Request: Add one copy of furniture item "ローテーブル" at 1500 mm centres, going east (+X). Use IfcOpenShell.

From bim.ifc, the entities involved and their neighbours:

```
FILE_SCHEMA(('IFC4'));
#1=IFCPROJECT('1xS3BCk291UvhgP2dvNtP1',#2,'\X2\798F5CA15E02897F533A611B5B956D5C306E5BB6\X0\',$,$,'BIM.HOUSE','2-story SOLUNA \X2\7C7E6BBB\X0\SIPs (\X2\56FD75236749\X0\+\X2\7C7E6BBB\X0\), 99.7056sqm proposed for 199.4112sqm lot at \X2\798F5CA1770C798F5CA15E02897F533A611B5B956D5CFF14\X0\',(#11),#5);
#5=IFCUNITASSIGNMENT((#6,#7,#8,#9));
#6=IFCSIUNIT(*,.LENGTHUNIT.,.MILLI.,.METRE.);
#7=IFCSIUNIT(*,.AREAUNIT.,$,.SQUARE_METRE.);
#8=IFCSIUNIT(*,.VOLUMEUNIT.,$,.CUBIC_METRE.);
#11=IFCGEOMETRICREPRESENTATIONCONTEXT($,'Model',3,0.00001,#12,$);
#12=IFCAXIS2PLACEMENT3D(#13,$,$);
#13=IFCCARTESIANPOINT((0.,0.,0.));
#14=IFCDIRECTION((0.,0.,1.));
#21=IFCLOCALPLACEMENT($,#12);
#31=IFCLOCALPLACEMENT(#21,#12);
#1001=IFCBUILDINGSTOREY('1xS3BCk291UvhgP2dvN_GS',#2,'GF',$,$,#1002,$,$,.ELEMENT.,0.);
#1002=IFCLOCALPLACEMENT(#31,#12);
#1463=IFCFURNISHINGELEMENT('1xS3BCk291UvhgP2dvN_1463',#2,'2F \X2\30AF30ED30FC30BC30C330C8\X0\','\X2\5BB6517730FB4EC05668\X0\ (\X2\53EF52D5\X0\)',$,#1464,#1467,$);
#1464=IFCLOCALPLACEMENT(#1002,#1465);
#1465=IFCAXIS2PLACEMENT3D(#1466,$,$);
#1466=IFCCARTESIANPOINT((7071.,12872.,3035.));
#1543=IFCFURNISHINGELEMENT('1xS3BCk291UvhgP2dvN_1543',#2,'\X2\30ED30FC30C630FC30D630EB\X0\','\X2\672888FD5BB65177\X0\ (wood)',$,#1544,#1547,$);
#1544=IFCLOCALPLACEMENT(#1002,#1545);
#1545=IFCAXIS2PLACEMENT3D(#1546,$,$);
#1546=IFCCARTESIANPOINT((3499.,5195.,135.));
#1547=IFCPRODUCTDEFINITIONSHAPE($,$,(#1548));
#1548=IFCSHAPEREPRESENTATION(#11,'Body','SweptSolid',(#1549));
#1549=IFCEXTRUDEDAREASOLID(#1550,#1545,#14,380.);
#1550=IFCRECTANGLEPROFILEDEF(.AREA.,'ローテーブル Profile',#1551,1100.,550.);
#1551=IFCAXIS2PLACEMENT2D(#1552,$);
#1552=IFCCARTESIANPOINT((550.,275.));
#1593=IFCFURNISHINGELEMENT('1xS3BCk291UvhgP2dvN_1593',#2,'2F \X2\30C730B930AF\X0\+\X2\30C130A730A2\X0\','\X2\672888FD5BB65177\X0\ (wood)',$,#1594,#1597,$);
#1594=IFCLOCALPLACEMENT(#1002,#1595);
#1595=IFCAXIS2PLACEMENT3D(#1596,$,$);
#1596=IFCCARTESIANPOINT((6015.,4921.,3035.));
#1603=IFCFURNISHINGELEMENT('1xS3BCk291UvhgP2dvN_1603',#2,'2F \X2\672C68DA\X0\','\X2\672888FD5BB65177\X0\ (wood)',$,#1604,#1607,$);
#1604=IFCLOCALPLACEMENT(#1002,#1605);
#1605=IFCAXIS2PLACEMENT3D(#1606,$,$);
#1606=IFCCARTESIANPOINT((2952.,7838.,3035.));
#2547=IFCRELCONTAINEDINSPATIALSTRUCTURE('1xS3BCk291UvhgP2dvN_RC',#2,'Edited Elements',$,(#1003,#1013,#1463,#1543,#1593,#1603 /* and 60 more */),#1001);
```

```python
import numpy as np
import ifcopenshell
import ifcopenshell.api.geometry
import ifcopenshell.api.root
import ifcopenshell.util.element
import ifcopenshell.util.placement

model = ifcopenshell.open("bim.ifc")


def reuse_history(source, copy):
    """copy_class also copies each property set's owner history, people and application; keep the originals."""
    for rel in copy.IsDefinedBy:
        if rel.is_a("IfcRelDefinesByProperties") and (history := rel.RelatingPropertyDefinition.OwnerHistory):
            rel.RelatingPropertyDefinition.OwnerHistory = source.OwnerHistory
            ifcopenshell.util.element.remove_deep2(model, history)


source = model.by_guid("1xS3BCk291UvhgP2dvN_1543")
base = ifcopenshell.util.placement.get_local_placement(source.ObjectPlacement)
step = np.array([1.0, 0.0, 0.0]) * 1500.0

for i in range(1, 2):
    copy = ifcopenshell.api.root.copy_class(model, product=source)
    copy.Representation = ifcopenshell.util.element.copy_deep(
        model, source.Representation, exclude=["IfcGeometricRepresentationContext", "IfcRepresentationMap"]
    )
    reuse_history(source, copy)
    matrix = base.copy()
    matrix[:3, 3] += i * step
    print("added at", matrix[:3, 3].round(3) + 0.0)
    ifcopenshell.api.geometry.edit_object_placement(model, product=copy, matrix=matrix, is_si=False)

model.write("bim-out.ifc")
```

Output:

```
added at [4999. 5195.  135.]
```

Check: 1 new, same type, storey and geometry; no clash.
